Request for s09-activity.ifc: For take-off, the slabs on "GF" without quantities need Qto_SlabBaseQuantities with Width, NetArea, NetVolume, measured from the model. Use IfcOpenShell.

First a look at what the model holds.

```python
import ifcopenshell
import ifcopenshell.util.element
import ifcopenshell.util.unit

model = ifcopenshell.open("s09-activity.ifc")
print(model.schema)
for unit_type in ("LENGTHUNIT", "AREAUNIT", "VOLUMEUNIT"):
    print(unit_type, ifcopenshell.util.unit.calculate_unit_scale(model, unit_type))
storey = next(s for s in model.by_type("IfcBuildingStorey") if s.Name == "GF")
slabs = [e for e in ifcopenshell.util.element.get_decomposition(storey) if e.is_a("IfcSlab")]
for e in sorted(slabs, key=lambda e: e.id()):
    print(e.id(), e.is_a(), e.Name, list(ifcopenshell.util.element.get_psets(e, qtos_only=True)), sep=" | ")
```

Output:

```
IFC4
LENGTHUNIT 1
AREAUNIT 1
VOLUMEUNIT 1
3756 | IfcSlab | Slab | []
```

```python
import ifcopenshell
import ifcopenshell.api.pset
import ifcopenshell.geom
import ifcopenshell.util.element
import ifcopenshell.util.shape
import ifcopenshell.util.unit

model = ifcopenshell.open("s09-activity.ifc")
unit_scale = ifcopenshell.util.unit.calculate_unit_scale(model)
area_scale = ifcopenshell.util.unit.calculate_unit_scale(model, "AREAUNIT")
volume_scale = ifcopenshell.util.unit.calculate_unit_scale(model, "VOLUMEUNIT")
settings = ifcopenshell.geom.settings()

storey = next(s for s in model.by_type("IfcBuildingStorey") if s.Name == "GF")
slabs = [e for e in ifcopenshell.util.element.get_decomposition(storey) if e.is_a("IfcSlab")]

for e in sorted(slabs, key=lambda e: e.id()):
    if ifcopenshell.util.element.get_psets(e, qtos_only=True, should_inherit=False):
        continue
    # Geometry comes back in metres, in the element's own axes.
    shape = ifcopenshell.geom.create_shape(settings, e)
    values = {
        "Width": ifcopenshell.util.shape.get_z(shape.geometry) / unit_scale,
        "NetArea": ifcopenshell.util.shape.get_footprint_area(shape.geometry) / area_scale,
        "NetVolume": ifcopenshell.util.shape.get_volume(shape.geometry) / volume_scale,
    }
    qto = ifcopenshell.api.pset.add_qto(model, product=e, name="Qto_SlabBaseQuantities")
    ifcopenshell.api.pset.edit_qto(model, qto=qto, properties=values)
    print(e.id(), {k: round(v, 3) for k, v in values.items()})

model.write("s09-activity-out.ifc")
```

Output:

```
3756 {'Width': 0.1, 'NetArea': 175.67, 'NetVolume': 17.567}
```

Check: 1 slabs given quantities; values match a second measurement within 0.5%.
